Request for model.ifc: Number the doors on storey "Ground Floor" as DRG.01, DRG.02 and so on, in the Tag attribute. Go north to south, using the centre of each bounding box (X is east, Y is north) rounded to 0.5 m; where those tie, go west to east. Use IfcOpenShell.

First a look at what the model holds.

```python
import ifcopenshell
import ifcopenshell.util.element
import ifcopenshell.util.placement

model = ifcopenshell.open("model.ifc")
print(model.schema)
storey = next(s for s in model.by_type("IfcBuildingStorey") if s.Name == "Ground Floor")
doors = [e for e in ifcopenshell.util.element.get_decomposition(storey) if e.is_a("IfcDoor")]
for e in sorted(doors, key=lambda e: e.id()):
    origin = ifcopenshell.util.placement.get_local_placement(e.ObjectPlacement)[:3, 3]
    print(e.id(), e.Tag, e.Name, origin.round(2) + 0.0, sep=" | ")
```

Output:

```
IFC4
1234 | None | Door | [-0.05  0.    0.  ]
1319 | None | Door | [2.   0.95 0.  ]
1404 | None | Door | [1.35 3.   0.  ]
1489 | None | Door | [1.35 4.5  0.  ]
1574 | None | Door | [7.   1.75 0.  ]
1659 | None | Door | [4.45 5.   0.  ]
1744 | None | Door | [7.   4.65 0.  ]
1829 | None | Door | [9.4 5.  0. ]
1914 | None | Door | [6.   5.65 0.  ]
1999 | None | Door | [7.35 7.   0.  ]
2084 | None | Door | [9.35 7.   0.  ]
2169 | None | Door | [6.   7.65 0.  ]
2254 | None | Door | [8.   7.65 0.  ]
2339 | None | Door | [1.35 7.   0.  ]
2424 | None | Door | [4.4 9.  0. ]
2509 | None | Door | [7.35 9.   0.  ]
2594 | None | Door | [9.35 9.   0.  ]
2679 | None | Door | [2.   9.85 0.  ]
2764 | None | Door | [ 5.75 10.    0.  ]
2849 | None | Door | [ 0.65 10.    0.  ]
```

```python
import ifcopenshell
import ifcopenshell.geom
import ifcopenshell.util.element
import ifcopenshell.util.shape

model = ifcopenshell.open("model.ifc")
settings = ifcopenshell.geom.settings()
settings.set("use-world-coords", True)


def centre(element):
    shape = ifcopenshell.geom.create_shape(settings, element)
    return ifcopenshell.util.shape.get_bbox_centroid(shape.geometry)


storey = next(s for s in model.by_type("IfcBuildingStorey") if s.Name == "Ground Floor")
doors = [e for e in ifcopenshell.util.element.get_decomposition(storey) if e.is_a("IfcDoor")]

# Insertion points can sit at a corner or the storey origin, so sort by the geometry (in metres).
centres = {e: centre(e) for e in doors}
doors.sort(key=lambda e: (-round(centres[e][1] / 0.5), centres[e][0]))

for i, e in enumerate(doors, start=1):
    number = f"DRG.{i:02d}"
    e.Tag = number
    print(e.id(), number)

model.write("model_rev.ifc")
```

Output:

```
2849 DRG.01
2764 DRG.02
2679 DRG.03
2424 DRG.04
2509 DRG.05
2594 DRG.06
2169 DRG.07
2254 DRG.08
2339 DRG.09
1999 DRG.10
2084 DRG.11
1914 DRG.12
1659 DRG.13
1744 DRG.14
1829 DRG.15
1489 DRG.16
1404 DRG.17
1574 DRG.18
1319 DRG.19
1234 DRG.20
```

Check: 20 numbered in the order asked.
